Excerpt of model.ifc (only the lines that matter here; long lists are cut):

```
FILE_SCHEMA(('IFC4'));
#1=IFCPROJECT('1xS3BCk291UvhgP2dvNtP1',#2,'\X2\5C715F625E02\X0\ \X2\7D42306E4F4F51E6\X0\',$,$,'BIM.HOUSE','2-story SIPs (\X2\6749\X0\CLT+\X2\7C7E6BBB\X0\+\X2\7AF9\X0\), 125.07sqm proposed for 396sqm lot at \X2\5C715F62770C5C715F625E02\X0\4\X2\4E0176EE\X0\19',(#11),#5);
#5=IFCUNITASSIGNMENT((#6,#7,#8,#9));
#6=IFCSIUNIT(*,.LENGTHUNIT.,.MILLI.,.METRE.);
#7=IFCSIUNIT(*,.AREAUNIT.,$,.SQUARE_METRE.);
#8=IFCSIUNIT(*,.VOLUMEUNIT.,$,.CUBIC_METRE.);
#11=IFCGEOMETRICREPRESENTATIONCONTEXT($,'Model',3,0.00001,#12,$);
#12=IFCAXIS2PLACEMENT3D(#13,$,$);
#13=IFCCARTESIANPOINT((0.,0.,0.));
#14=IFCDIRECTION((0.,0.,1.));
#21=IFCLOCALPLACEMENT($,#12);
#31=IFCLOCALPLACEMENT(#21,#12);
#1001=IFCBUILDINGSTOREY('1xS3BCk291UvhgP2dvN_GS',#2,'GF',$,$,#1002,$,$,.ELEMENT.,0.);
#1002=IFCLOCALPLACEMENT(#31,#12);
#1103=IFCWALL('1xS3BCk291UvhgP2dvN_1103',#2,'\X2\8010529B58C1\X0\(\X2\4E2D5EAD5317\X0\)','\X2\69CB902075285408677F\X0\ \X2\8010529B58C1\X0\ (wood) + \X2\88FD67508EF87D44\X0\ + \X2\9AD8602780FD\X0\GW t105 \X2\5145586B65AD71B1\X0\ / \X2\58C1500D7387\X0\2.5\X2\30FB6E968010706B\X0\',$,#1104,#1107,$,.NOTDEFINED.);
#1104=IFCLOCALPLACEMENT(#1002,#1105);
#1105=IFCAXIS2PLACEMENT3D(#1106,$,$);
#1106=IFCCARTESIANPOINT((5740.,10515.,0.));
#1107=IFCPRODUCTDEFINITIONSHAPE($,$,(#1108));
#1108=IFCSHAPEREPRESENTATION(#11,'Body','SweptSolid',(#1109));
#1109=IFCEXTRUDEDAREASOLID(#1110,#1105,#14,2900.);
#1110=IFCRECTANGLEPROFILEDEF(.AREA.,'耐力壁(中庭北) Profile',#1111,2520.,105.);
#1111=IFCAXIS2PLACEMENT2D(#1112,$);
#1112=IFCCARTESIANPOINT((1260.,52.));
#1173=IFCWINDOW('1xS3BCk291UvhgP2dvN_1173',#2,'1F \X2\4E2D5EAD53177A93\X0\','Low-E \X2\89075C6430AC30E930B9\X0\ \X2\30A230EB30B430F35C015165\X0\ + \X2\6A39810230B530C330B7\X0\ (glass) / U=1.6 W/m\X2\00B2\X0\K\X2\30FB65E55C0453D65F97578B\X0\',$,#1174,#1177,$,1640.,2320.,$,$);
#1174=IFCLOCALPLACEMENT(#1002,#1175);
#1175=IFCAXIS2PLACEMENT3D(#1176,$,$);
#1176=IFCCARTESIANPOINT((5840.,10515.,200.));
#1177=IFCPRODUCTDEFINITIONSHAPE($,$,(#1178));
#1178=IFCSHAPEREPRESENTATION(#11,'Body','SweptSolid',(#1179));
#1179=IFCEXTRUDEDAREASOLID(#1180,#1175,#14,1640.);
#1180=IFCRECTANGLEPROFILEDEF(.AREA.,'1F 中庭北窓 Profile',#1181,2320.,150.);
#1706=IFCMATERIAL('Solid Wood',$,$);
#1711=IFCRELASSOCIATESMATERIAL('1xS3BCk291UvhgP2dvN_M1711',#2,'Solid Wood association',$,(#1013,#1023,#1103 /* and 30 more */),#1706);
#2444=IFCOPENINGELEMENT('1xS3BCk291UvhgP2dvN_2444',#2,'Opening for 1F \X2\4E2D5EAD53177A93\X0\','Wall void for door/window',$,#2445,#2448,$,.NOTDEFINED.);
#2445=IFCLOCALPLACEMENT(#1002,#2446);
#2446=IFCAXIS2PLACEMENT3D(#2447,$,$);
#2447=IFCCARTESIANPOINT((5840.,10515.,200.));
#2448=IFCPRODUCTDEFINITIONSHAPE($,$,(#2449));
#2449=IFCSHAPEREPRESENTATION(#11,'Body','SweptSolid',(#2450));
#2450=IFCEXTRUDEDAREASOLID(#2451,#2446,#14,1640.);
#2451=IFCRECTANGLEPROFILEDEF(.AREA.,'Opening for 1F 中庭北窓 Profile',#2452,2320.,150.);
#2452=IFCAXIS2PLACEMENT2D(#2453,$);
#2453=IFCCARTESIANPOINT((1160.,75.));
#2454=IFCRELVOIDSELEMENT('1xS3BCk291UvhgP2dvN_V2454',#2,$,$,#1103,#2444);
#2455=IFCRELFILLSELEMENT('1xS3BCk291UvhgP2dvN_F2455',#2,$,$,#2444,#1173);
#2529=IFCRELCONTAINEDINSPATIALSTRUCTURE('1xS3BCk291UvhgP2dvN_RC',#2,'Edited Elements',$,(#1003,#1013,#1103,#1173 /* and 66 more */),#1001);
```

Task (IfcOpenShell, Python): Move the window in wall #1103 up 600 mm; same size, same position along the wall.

```python
import numpy as np
import ifcopenshell
import ifcopenshell.api.geometry
import ifcopenshell.util.placement
import ifcopenshell.util.unit

model = ifcopenshell.open("model.ifc")
unit_scale = ifcopenshell.util.unit.calculate_unit_scale(model)

window = model.by_guid("1xS3BCk291UvhgP2dvN_1173")
opening = window.FillsVoids[0].RelatingOpeningElement
dz = 0.6 / unit_scale

shift = np.array([0.0, 0.0, dz])
# The window is not placed relative to its opening, so move both.
for product in (opening, window):
    matrix = ifcopenshell.util.placement.get_local_placement(product.ObjectPlacement)
    matrix[:3, 3] += shift
    ifcopenshell.api.geometry.edit_object_placement(model, product=product, matrix=matrix, is_si=False)

print(f"moved by {dz * unit_scale:+.3f} m")

model.write("model_rev.ifc")
```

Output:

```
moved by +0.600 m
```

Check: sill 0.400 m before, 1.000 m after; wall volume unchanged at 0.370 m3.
